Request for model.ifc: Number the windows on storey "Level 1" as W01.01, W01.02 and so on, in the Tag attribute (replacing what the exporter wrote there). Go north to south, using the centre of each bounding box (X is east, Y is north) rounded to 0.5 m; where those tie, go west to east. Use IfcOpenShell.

First a look at what the model holds.

```python
import ifcopenshell
import ifcopenshell.util.element
import ifcopenshell.util.placement

model = ifcopenshell.open("model.ifc")
print(model.schema)
storey = next(s for s in model.by_type("IfcBuildingStorey") if s.Name == "Level 1")
windows = [e for e in ifcopenshell.util.element.get_decomposition(storey) if e.is_a("IfcWindow")]
for e in sorted(windows, key=lambda e: e.id()):
    origin = ifcopenshell.util.placement.get_local_placement(e.ObjectPlacement)[:3, 3]
    print(e.id(), e.Tag, e.Name, origin.round(2) + 0.0, sep=" | ")
```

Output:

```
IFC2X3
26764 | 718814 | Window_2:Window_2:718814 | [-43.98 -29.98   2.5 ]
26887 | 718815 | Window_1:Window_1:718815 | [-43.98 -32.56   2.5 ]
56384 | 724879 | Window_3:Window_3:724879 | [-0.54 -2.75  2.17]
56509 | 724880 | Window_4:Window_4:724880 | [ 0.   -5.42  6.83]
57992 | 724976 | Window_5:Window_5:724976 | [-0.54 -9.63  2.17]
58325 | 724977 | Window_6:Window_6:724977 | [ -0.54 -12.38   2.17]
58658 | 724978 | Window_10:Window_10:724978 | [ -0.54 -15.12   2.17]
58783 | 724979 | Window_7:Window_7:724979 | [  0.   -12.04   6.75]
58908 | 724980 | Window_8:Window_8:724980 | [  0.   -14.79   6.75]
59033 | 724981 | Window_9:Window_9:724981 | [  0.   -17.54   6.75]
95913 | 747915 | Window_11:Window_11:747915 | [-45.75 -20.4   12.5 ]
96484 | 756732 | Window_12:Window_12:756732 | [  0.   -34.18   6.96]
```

```python
import ifcopenshell
import ifcopenshell.geom
import ifcopenshell.util.element
import ifcopenshell.util.shape

model = ifcopenshell.open("model.ifc")
settings = ifcopenshell.geom.settings()
settings.set("use-world-coords", True)


def centre(element):
    shape = ifcopenshell.geom.create_shape(settings, element)
    return ifcopenshell.util.shape.get_bbox_centroid(shape.geometry)


storey = next(s for s in model.by_type("IfcBuildingStorey") if s.Name == "Level 1")
windows = [e for e in ifcopenshell.util.element.get_decomposition(storey) if e.is_a("IfcWindow")]

# Insertion points can sit at a corner or the storey origin, so sort by the geometry (in metres).
centres = {e: centre(e) for e in windows}
windows.sort(key=lambda e: (-round(centres[e][1] / 0.5), centres[e][0]))

for i, e in enumerate(windows, start=1):
    number = f"W01.{i:02d}"
    e.Tag = number
    print(e.id(), number)

model.write("model_updated.ifc")
```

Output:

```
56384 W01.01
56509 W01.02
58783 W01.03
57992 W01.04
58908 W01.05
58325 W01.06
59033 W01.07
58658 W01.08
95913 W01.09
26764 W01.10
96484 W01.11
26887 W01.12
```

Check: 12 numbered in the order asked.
